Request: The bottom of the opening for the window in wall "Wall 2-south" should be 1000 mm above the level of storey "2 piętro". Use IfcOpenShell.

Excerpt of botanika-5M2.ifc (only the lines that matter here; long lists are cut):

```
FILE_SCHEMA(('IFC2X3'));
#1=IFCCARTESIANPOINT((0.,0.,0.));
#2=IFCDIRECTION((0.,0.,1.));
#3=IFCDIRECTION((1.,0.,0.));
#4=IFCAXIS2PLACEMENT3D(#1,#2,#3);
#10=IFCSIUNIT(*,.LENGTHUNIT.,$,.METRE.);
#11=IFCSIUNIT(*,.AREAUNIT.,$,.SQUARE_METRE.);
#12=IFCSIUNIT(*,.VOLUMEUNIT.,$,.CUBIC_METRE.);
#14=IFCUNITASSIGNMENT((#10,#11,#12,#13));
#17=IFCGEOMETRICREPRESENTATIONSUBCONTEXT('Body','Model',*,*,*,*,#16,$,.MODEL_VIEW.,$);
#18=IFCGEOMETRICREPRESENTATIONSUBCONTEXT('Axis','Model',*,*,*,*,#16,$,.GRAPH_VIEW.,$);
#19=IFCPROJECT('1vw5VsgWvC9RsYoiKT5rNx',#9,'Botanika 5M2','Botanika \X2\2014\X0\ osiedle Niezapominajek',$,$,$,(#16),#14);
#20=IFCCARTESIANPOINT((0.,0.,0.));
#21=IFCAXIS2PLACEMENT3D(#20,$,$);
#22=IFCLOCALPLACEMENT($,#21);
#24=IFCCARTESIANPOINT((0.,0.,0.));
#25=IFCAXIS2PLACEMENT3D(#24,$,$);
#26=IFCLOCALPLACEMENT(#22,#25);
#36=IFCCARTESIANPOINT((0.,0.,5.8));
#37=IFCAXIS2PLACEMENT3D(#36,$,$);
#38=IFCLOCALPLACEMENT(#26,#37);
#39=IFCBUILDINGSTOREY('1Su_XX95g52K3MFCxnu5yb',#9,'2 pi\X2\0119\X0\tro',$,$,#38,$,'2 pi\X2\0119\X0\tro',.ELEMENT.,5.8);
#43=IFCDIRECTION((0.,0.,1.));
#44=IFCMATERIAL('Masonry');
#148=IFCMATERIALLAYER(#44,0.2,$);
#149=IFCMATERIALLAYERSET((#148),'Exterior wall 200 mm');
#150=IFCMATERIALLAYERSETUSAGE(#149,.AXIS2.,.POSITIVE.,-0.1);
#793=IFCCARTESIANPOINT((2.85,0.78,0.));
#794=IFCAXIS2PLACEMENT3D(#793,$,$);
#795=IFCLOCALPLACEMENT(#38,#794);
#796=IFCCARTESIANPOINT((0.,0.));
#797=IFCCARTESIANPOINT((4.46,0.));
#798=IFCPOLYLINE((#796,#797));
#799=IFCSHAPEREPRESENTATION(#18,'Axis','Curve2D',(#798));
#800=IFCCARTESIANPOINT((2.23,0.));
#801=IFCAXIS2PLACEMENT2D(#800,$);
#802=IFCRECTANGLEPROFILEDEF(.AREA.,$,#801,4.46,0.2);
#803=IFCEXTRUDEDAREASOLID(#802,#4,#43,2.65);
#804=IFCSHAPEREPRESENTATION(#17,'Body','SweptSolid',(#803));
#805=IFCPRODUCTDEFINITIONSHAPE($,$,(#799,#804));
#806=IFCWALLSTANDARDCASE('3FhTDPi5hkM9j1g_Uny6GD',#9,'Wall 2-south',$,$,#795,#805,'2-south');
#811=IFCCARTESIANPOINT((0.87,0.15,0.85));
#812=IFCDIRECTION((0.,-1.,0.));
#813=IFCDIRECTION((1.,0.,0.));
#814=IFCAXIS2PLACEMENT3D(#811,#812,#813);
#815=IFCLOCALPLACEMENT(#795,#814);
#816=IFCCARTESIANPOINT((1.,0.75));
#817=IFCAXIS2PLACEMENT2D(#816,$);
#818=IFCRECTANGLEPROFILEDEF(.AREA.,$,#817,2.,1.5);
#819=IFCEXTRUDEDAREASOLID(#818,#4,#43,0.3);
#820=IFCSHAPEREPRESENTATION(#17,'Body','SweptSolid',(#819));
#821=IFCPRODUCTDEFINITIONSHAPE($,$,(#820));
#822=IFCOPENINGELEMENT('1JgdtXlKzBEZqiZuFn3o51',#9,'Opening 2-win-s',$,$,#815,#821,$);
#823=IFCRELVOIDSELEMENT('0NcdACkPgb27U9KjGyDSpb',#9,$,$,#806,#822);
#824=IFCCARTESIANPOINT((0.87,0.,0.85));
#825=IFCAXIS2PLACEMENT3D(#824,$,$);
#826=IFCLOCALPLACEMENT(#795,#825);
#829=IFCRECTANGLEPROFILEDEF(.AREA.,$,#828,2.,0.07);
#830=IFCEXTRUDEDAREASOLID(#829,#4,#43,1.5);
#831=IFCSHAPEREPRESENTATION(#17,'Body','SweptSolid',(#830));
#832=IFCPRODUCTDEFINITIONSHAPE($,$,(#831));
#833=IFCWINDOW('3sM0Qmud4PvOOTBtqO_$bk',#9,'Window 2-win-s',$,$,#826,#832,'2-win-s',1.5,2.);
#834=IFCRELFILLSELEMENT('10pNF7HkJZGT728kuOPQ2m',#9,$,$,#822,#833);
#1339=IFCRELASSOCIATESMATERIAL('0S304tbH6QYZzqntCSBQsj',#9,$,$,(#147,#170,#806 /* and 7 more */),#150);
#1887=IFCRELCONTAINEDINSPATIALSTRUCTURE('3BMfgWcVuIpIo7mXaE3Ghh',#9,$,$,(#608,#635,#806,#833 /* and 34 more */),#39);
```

```python
import numpy as np
import ifcopenshell
import ifcopenshell.api.geometry
import ifcopenshell.geom
import ifcopenshell.util.element
import ifcopenshell.util.placement
import ifcopenshell.util.shape
import ifcopenshell.util.unit

model = ifcopenshell.open("botanika-5M2.ifc")
unit_scale = ifcopenshell.util.unit.calculate_unit_scale(model)

window = model.by_guid("3sM0Qmud4PvOOTBtqO_$bk")
opening = window.FillsVoids[0].RelatingOpeningElement
storey = ifcopenshell.util.element.get_container(window, ifc_class="IfcBuildingStorey")
level = ifcopenshell.util.placement.get_local_placement(storey.ObjectPlacement)[2, 3]

# The opening's origin need not be at the sill, so measure its lowest point.
shape = ifcopenshell.geom.create_shape(ifcopenshell.geom.settings(), opening)
bottom = ifcopenshell.util.shape.get_shape_bottom_elevation(shape, shape.geometry) / unit_scale
dz = level + 1 / unit_scale - bottom

shift = np.array([0.0, 0.0, dz])
# The window is not placed relative to its opening, so move both.
for product in (opening, window):
    matrix = ifcopenshell.util.placement.get_local_placement(product.ObjectPlacement)
    matrix[:3, 3] += shift
    ifcopenshell.api.geometry.edit_object_placement(model, product=product, matrix=matrix, is_si=False)

print(f"moved by {dz * unit_scale:+.3f} m")

model.write("botanika-5M2_updated.ifc")
```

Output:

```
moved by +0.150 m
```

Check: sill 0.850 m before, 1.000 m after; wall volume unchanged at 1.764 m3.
